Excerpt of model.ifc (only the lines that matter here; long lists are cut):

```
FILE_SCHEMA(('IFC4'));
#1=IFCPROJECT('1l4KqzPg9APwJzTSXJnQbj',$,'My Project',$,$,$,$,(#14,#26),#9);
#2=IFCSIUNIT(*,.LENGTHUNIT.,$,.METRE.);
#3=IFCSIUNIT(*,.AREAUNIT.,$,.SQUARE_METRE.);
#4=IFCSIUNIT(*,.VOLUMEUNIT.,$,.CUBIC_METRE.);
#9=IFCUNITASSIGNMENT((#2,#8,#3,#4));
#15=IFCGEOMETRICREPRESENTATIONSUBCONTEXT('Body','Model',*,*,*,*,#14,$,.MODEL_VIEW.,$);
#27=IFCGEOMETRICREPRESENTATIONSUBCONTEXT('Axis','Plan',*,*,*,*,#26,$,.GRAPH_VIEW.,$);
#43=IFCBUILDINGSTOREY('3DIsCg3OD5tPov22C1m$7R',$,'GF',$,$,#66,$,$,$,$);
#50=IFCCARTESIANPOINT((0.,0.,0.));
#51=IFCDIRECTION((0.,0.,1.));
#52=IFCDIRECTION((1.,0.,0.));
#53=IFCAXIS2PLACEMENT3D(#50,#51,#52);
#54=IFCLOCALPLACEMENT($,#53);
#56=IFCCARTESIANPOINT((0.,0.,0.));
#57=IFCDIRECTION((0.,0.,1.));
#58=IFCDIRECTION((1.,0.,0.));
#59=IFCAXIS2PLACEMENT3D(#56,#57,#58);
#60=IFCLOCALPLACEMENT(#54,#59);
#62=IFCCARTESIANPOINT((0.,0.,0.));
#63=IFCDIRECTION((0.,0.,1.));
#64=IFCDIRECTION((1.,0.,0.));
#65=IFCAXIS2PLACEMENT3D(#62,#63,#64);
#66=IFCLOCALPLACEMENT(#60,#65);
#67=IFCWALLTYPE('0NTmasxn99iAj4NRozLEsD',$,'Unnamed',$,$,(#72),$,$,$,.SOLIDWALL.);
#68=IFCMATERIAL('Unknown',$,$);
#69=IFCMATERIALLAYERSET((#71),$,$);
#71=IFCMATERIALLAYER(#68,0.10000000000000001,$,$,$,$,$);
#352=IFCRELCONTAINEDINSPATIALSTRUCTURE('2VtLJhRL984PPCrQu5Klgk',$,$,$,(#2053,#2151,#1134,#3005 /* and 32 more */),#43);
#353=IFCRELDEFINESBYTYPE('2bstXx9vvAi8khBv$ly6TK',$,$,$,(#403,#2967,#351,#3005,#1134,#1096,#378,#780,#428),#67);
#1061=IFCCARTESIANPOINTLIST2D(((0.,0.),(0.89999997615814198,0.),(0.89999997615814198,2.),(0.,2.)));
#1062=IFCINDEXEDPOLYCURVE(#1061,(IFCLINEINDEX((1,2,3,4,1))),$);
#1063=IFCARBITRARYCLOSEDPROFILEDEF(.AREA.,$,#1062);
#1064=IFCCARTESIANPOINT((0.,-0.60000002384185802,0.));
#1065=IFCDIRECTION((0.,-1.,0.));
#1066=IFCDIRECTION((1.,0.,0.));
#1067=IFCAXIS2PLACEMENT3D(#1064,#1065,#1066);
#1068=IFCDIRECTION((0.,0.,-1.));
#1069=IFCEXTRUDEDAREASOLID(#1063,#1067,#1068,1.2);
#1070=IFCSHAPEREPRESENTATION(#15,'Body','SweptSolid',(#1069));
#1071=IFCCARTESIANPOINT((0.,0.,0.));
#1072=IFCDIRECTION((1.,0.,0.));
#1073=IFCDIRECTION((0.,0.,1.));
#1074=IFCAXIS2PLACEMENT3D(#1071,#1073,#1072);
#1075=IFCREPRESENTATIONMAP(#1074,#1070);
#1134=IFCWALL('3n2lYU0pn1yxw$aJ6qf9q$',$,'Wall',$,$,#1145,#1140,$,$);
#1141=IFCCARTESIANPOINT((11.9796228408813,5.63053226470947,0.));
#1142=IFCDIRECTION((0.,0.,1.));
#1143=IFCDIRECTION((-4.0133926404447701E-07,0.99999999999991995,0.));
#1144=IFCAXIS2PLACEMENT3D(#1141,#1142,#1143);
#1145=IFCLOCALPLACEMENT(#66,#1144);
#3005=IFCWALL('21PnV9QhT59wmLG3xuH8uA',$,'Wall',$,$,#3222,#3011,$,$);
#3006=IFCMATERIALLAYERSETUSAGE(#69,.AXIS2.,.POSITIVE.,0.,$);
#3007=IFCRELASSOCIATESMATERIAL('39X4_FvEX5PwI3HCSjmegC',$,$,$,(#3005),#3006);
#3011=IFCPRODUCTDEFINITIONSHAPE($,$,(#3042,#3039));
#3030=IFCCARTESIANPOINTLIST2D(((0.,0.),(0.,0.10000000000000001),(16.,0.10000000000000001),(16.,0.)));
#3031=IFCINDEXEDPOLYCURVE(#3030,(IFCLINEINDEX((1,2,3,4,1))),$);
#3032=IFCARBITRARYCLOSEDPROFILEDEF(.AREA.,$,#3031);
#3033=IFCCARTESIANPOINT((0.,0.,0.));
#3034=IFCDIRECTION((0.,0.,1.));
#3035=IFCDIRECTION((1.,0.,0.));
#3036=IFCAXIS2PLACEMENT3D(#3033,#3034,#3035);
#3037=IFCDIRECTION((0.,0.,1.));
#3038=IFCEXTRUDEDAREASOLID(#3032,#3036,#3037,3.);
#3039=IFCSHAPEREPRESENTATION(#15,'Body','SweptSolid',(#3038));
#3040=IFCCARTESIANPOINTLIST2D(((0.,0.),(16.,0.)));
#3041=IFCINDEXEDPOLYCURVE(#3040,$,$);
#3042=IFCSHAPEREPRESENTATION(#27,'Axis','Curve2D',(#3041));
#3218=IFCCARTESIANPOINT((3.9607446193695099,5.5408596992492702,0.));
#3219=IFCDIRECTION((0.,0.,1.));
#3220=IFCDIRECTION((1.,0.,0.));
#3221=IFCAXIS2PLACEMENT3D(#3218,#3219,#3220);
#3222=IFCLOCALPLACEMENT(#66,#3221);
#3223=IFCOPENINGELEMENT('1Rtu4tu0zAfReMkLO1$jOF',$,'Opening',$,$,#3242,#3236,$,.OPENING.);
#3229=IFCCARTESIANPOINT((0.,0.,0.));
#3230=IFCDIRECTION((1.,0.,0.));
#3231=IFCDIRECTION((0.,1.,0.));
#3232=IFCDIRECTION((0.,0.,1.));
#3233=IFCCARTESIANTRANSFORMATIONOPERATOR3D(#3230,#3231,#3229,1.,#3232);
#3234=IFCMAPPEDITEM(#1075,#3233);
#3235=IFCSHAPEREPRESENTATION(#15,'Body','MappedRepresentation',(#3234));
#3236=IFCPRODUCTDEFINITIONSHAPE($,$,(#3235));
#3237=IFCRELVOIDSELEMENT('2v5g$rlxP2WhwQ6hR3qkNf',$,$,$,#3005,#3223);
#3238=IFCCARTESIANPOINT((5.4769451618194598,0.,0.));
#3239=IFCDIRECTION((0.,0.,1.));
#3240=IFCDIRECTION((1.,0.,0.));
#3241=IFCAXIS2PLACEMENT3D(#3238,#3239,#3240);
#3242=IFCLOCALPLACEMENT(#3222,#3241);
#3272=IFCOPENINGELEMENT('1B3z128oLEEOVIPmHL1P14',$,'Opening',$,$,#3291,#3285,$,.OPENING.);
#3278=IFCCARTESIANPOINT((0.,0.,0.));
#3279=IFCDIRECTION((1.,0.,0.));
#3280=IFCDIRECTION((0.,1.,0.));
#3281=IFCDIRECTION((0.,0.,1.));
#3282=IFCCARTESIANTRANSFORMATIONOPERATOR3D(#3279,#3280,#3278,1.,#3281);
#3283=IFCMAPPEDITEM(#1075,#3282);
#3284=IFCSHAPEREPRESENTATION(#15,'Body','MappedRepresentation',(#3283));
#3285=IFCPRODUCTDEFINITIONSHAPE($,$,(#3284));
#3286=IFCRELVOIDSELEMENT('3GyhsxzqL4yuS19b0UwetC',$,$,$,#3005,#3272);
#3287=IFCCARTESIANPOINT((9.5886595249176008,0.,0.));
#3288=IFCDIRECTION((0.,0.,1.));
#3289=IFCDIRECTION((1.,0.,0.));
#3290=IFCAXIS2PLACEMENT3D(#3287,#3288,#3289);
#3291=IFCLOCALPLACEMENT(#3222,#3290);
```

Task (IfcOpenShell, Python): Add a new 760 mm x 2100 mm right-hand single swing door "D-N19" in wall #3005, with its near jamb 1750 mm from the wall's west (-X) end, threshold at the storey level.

```python
import numpy as np
import ifcopenshell
import ifcopenshell.api.feature
import ifcopenshell.api.geometry
import ifcopenshell.api.root
import ifcopenshell.api.spatial
import ifcopenshell.geom
import ifcopenshell.util.element
import ifcopenshell.util.placement
import ifcopenshell.util.representation
import ifcopenshell.util.shape
import ifcopenshell.util.unit

model = ifcopenshell.open("model.ifc")
unit_scale = ifcopenshell.util.unit.calculate_unit_scale(model)
settings = ifcopenshell.geom.settings()


def volume(element):
    """Net volume in cubic metres, openings subtracted."""
    shape = ifcopenshell.geom.create_shape(settings, element)
    return ifcopenshell.util.shape.get_volume(shape.geometry)


wall = model.by_guid("21PnV9QhT59wmLG3xuH8uA")
storey = ifcopenshell.util.element.get_container(wall, ifc_class="IfcBuildingStorey")
context = ifcopenshell.util.representation.get_context(model, "Model", "Body", "MODEL_VIEW")
before = volume(wall)

width, height, from_end, sill = 0.76, 2.1, 1.75, 0.0  # metres

# The wall runs along its own X axis, and the end named is its -X end.
wall_shape = ifcopenshell.geom.create_shape(settings, wall)
x, y, z = ifcopenshell.util.shape.get_vertices(wall_shape.geometry).T
start = x.min() + from_end
face, thickness = float(y.min()), float(y.max() - y.min())
wall_matrix = ifcopenshell.util.placement.get_local_placement(wall.ObjectPlacement)
level = ifcopenshell.util.placement.get_local_placement(storey.ObjectPlacement)[2, 3]


def in_wall(x, y):
    """Placement at x, y metres in the wall's axes, at sill height."""
    matrix = wall_matrix.copy()
    matrix[:, 3] = wall_matrix @ np.array([x / unit_scale, y / unit_scale, 0.0, 1.0])
    matrix[2, 3] = level + sill / unit_scale
    return matrix


# Opening: a box that overshoots both wall faces by 50 mm.
opening = ifcopenshell.api.root.create_entity(model, ifc_class="IfcOpeningElement", predefined_type="OPENING")
box = ifcopenshell.api.geometry.add_wall_representation(
    model, context=context, length=width, height=height, thickness=thickness + 0.1
)
ifcopenshell.api.geometry.assign_representation(model, product=opening, representation=box)
ifcopenshell.api.geometry.edit_object_placement(model, product=opening, matrix=in_wall(start, face - 0.05), is_si=False)
ifcopenshell.api.feature.add_feature(model, feature=opening, element=wall)

door = ifcopenshell.api.root.create_entity(model, ifc_class="IfcDoor", name="D-N19", predefined_type="DOOR")
door.OverallWidth, door.OverallHeight = width / unit_scale, height / unit_scale
door.OperationType = "SINGLE_SWING_RIGHT"
body = ifcopenshell.api.geometry.add_door_representation(
    model,
    context=context,
    overall_width=door.OverallWidth,
    overall_height=door.OverallHeight,
    operation_type="SINGLE_SWING_RIGHT",
    lining_properties={"LiningDepth": thickness / unit_scale, "ThresholdDepth": thickness / unit_scale},
)
ifcopenshell.api.geometry.assign_representation(model, product=door, representation=body)
ifcopenshell.api.spatial.assign_container(model, products=[door], relating_structure=storey)
ifcopenshell.api.feature.add_filling(model, opening=opening, element=door)

# The lining spans the wall, so the door starts at the wall face.
ifcopenshell.api.geometry.edit_object_placement(model, product=door, matrix=in_wall(start, face), is_si=False)

after = volume(wall)

print(f"wall volume {before:.3f} -> {after:.3f} m3")

model.write("model_edited.ifc")
```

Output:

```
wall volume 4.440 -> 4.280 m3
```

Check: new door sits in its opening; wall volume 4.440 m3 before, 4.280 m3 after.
